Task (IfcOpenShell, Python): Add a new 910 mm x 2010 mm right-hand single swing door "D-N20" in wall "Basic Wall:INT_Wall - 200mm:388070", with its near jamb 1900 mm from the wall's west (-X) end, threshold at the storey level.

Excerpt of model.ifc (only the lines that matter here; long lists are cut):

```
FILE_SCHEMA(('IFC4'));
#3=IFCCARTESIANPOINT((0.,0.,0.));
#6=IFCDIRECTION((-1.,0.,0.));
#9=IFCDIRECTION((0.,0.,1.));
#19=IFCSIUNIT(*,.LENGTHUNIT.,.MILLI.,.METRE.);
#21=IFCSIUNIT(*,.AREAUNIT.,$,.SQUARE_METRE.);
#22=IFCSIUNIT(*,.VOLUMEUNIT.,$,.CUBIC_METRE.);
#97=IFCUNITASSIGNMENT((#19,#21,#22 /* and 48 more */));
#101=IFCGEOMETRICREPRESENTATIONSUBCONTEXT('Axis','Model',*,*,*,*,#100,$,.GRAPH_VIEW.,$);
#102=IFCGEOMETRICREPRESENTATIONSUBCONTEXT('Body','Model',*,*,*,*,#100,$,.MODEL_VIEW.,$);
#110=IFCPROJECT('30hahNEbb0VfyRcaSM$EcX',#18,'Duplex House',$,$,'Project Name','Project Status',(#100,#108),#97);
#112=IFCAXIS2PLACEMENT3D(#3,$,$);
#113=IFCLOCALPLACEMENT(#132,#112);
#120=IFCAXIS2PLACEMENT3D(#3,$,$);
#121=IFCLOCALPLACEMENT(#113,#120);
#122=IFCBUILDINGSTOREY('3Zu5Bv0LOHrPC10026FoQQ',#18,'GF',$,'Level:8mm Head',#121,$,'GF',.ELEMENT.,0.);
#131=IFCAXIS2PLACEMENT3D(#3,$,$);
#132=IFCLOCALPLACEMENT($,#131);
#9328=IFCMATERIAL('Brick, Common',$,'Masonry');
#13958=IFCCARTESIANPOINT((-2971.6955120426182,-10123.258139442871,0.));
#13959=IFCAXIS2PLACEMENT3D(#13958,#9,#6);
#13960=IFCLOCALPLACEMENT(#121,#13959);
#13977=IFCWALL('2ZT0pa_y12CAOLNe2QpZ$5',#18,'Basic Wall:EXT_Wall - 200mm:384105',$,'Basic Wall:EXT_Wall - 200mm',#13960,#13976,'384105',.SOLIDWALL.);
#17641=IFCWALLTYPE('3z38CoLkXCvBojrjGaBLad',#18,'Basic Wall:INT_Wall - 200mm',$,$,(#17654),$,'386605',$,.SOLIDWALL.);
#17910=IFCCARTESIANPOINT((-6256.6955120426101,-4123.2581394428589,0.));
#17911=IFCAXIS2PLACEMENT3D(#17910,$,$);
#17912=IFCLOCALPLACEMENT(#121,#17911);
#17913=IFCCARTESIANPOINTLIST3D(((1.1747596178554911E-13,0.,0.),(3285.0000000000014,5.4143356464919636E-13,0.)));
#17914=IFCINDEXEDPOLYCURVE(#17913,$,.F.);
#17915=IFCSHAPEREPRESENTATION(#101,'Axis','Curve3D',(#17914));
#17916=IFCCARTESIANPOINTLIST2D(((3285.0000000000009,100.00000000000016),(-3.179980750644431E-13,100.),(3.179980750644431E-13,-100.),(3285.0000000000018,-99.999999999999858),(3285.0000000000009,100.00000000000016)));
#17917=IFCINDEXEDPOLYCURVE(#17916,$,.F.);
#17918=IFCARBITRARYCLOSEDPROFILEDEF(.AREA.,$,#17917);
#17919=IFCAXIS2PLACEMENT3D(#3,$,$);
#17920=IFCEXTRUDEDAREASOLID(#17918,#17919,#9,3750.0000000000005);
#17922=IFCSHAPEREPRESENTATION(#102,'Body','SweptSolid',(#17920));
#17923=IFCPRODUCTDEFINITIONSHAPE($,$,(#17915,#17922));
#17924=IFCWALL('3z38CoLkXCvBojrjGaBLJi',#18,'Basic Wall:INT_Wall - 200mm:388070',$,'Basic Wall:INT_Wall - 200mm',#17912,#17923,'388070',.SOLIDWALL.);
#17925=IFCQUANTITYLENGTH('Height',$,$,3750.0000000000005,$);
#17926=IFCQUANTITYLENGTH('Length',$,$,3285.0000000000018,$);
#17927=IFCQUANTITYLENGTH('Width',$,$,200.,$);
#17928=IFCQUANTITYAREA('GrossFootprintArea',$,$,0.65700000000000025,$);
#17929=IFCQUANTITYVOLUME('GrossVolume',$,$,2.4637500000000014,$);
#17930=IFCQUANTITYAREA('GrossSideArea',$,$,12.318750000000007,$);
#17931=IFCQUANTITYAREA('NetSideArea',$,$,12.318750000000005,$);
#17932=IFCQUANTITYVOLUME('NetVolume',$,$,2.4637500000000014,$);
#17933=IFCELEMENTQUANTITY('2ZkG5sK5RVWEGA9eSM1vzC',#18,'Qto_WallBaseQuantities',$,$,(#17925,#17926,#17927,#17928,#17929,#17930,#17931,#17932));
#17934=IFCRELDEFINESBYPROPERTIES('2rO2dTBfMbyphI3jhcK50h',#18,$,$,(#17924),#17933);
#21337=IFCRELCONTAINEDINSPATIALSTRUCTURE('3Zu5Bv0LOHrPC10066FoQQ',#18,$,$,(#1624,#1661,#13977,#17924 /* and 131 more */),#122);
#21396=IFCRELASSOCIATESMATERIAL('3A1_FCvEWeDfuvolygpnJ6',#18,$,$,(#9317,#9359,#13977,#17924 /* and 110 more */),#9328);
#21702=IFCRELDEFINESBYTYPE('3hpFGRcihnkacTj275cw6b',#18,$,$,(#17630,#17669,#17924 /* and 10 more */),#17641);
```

```python
import numpy as np
import ifcopenshell
import ifcopenshell.api.feature
import ifcopenshell.api.geometry
import ifcopenshell.api.pset
import ifcopenshell.api.root
import ifcopenshell.api.spatial
import ifcopenshell.geom
import ifcopenshell.util.element
import ifcopenshell.util.placement
import ifcopenshell.util.representation
import ifcopenshell.util.shape
import ifcopenshell.util.unit

model = ifcopenshell.open("model.ifc")
unit_scale = ifcopenshell.util.unit.calculate_unit_scale(model)
area_scale = ifcopenshell.util.unit.calculate_unit_scale(model, "AREAUNIT")
volume_scale = ifcopenshell.util.unit.calculate_unit_scale(model, "VOLUMEUNIT")
settings = ifcopenshell.geom.settings()


def volume(element):
    """Net volume in cubic metres, openings subtracted."""
    shape = ifcopenshell.geom.create_shape(settings, element)
    return ifcopenshell.util.shape.get_volume(shape.geometry)


wall = model.by_guid("3z38CoLkXCvBojrjGaBLJi")
storey = ifcopenshell.util.element.get_container(wall, ifc_class="IfcBuildingStorey")
context = ifcopenshell.util.representation.get_context(model, "Model", "Body", "MODEL_VIEW")
before = volume(wall)

width, height, from_end, sill = 0.91, 2.01, 1.9, 0.0  # metres

# The wall runs along its own X axis, and the end named is its -X end.
wall_shape = ifcopenshell.geom.create_shape(settings, wall)
x, y, z = ifcopenshell.util.shape.get_vertices(wall_shape.geometry).T
start = x.min() + from_end
face, thickness = float(y.min()), float(y.max() - y.min())
wall_matrix = ifcopenshell.util.placement.get_local_placement(wall.ObjectPlacement)
level = ifcopenshell.util.placement.get_local_placement(storey.ObjectPlacement)[2, 3]


def in_wall(x, y):
    """Placement at x, y metres in the wall's axes, at sill height."""
    matrix = wall_matrix.copy()
    matrix[:, 3] = wall_matrix @ np.array([x / unit_scale, y / unit_scale, 0.0, 1.0])
    matrix[2, 3] = level + sill / unit_scale
    return matrix


# Opening: a box that overshoots both wall faces by 50 mm.
opening = ifcopenshell.api.root.create_entity(model, ifc_class="IfcOpeningElement", predefined_type="OPENING")
box = ifcopenshell.api.geometry.add_wall_representation(
    model, context=context, length=width, height=height, thickness=thickness + 0.1
)
ifcopenshell.api.geometry.assign_representation(model, product=opening, representation=box)
ifcopenshell.api.geometry.edit_object_placement(model, product=opening, matrix=in_wall(start, face - 0.05), is_si=False)
ifcopenshell.api.feature.add_feature(model, feature=opening, element=wall)

door = ifcopenshell.api.root.create_entity(model, ifc_class="IfcDoor", name="D-N20", predefined_type="DOOR")
door.OverallWidth, door.OverallHeight = width / unit_scale, height / unit_scale
door.OperationType = "SINGLE_SWING_RIGHT"
body = ifcopenshell.api.geometry.add_door_representation(
    model,
    context=context,
    overall_width=door.OverallWidth,
    overall_height=door.OverallHeight,
    operation_type="SINGLE_SWING_RIGHT",
    lining_properties={"LiningDepth": thickness / unit_scale, "ThresholdDepth": thickness / unit_scale},
)
ifcopenshell.api.geometry.assign_representation(model, product=door, representation=body)
ifcopenshell.api.spatial.assign_container(model, products=[door], relating_structure=storey)
ifcopenshell.api.feature.add_filling(model, opening=opening, element=door)

# The lining spans the wall, so the door starts at the wall face.
ifcopenshell.api.geometry.edit_object_placement(model, product=door, matrix=in_wall(start, face), is_si=False)

after = volume(wall)

# Update the wall's stored quantities.
qto = model.by_id(ifcopenshell.util.element.get_pset(wall, "Qto_WallBaseQuantities", should_inherit=False)["id"])
ifcopenshell.api.pset.edit_qto(model, qto=qto, properties={
    "NetSideArea": after / thickness / area_scale,
    "NetVolume": after / volume_scale,
})

print(f"wall volume {before:.3f} -> {after:.3f} m3")

model.write("model-out.ifc")
```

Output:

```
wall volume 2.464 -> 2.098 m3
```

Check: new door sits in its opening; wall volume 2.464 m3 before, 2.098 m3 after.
